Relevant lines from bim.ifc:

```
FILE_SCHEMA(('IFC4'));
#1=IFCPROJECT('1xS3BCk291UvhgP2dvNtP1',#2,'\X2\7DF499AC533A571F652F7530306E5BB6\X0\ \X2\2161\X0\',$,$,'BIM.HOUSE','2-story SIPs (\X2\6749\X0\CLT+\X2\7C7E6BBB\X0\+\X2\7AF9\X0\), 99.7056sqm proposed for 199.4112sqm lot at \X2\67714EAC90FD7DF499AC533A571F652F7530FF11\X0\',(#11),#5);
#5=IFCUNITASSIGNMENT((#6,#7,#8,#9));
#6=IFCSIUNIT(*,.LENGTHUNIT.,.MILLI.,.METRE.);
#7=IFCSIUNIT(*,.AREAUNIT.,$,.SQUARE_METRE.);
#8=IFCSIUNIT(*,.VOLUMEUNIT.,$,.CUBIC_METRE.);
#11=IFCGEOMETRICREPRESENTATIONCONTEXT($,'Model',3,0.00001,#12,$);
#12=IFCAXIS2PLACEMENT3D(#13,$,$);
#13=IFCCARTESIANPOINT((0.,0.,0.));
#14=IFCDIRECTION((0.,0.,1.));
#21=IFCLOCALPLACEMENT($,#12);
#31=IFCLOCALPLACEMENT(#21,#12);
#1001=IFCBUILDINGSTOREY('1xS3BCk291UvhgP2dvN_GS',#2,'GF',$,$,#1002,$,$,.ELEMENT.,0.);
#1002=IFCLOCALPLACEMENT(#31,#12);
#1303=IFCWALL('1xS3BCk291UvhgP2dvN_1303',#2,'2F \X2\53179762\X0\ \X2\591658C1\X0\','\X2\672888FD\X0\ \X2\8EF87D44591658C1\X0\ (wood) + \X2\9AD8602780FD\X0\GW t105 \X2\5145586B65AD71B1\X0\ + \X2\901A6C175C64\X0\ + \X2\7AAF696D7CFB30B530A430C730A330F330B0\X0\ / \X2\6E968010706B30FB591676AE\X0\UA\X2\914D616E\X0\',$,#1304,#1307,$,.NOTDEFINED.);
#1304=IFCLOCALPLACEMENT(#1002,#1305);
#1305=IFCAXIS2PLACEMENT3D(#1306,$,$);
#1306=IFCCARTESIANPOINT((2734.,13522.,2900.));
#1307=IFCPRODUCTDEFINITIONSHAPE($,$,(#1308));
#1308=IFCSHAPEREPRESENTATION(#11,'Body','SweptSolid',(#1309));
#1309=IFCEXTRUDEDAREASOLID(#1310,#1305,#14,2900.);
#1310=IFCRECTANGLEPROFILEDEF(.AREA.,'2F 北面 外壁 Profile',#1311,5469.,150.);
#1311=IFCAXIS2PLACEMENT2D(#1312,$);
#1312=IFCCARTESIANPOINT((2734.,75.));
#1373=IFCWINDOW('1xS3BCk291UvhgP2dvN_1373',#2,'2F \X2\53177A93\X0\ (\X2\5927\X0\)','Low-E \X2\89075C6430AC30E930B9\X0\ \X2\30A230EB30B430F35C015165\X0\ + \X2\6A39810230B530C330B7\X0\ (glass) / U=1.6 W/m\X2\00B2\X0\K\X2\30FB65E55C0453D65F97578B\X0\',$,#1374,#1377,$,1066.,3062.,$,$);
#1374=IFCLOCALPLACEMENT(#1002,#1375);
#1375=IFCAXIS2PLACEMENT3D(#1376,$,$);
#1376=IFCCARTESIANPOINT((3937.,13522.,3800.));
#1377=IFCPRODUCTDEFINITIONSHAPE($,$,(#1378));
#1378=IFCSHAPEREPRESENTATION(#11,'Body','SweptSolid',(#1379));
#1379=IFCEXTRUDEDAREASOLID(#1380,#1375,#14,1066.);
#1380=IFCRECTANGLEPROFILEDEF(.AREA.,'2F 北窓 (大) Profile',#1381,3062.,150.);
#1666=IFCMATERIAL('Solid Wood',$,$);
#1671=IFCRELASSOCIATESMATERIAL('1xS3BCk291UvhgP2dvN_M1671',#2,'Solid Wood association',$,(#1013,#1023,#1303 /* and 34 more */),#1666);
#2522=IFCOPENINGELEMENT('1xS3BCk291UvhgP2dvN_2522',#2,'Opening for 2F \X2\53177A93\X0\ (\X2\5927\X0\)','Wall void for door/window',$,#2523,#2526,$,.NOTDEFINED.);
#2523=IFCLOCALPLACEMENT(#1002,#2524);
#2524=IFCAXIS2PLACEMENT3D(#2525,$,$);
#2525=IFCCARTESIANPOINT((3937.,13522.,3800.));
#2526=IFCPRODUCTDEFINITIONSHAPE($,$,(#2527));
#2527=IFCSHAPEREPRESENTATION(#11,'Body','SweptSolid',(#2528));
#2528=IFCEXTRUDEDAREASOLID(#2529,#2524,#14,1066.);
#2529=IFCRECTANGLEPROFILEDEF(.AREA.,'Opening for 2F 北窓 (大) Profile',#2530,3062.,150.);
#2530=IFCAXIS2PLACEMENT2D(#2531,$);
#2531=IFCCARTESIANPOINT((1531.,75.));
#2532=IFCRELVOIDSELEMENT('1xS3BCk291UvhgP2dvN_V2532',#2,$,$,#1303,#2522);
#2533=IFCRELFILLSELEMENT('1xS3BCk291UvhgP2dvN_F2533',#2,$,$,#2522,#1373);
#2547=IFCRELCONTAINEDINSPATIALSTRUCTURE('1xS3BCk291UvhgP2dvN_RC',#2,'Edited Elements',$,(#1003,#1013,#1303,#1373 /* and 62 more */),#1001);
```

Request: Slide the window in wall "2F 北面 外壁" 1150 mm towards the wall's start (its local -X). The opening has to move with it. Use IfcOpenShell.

```python
import ifcopenshell
import ifcopenshell.api.geometry
import ifcopenshell.util.placement
import ifcopenshell.util.unit

model = ifcopenshell.open("bim.ifc")
unit_scale = ifcopenshell.util.unit.calculate_unit_scale(model)

window = model.by_id(1373)
opening = window.FillsVoids[0].RelatingOpeningElement
wall = opening.VoidsElements[0].RelatingBuildingElement

wall_matrix = ifcopenshell.util.placement.get_local_placement(wall.ObjectPlacement)
shift = wall_matrix[:3, 0] * -1.15 / unit_scale
before = ifcopenshell.util.placement.get_local_placement(window.ObjectPlacement)[:3, 3].copy()

# The window is not placed relative to its opening, so move both.
for product in (opening, window):
    matrix = ifcopenshell.util.placement.get_local_placement(product.ObjectPlacement)
    matrix[:3, 3] += shift
    ifcopenshell.api.geometry.edit_object_placement(model, product=product, matrix=matrix, is_si=False)

after = ifcopenshell.util.placement.get_local_placement(window.ObjectPlacement)[:3, 3]
print("window moved by", (after - before).round(3) + 0.0)

model.write("bim_updated.ifc")
```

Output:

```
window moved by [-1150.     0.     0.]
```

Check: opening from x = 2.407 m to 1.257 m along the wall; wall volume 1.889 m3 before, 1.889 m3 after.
